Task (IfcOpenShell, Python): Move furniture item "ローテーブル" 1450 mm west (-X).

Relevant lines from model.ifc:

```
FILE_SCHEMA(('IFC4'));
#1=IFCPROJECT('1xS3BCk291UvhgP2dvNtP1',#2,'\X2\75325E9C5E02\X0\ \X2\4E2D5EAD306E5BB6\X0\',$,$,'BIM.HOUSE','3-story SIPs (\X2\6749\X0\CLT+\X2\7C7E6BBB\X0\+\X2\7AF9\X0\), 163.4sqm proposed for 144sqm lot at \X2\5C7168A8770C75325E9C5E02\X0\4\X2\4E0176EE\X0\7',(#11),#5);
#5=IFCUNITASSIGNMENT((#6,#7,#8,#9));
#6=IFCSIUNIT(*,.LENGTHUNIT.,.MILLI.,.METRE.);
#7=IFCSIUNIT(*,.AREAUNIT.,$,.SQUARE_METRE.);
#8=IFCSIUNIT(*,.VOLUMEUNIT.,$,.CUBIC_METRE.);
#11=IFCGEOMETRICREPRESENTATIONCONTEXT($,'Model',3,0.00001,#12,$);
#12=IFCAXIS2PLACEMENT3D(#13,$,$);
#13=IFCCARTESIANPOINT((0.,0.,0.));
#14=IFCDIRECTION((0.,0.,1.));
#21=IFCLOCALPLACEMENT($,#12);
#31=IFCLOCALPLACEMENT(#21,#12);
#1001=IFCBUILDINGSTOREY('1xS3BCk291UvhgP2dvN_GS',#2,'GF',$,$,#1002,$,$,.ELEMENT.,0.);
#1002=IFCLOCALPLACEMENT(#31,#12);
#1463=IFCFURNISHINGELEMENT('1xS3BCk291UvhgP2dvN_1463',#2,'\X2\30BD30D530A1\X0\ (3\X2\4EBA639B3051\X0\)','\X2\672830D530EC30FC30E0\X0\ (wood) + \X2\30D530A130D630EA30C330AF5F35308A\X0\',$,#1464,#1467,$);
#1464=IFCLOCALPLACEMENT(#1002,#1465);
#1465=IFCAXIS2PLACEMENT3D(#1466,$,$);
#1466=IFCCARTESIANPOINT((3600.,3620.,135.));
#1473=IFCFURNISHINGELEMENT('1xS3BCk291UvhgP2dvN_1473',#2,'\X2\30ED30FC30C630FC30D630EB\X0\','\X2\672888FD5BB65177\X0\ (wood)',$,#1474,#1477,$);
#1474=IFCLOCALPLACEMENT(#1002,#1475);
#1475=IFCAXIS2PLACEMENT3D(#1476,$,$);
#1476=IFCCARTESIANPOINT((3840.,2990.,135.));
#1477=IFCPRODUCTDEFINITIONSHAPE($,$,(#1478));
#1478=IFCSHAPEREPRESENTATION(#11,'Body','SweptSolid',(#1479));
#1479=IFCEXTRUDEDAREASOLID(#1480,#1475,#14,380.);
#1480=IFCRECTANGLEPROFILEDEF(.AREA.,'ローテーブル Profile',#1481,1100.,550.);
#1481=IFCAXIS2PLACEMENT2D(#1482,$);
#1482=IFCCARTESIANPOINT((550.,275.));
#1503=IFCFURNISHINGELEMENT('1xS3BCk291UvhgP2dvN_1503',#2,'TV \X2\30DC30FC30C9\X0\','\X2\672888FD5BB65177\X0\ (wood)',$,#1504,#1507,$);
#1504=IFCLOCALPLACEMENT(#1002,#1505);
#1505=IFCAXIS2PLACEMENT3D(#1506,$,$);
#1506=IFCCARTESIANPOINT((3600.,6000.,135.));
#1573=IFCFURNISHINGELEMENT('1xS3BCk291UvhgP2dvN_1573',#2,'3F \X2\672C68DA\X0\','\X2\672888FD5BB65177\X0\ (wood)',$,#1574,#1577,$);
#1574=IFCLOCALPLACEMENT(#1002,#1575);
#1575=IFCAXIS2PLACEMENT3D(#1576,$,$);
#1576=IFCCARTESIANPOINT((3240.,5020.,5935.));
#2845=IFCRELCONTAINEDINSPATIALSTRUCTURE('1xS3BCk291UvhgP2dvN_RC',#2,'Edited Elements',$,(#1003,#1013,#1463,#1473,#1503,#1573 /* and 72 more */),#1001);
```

```python
import ifcopenshell
import ifcopenshell.api.geometry
import ifcopenshell.util.placement
import ifcopenshell.util.unit

model = ifcopenshell.open("model.ifc")
unit_scale = ifcopenshell.util.unit.calculate_unit_scale(model)

item = model.by_guid("1xS3BCk291UvhgP2dvN_1473")
matrix = ifcopenshell.util.placement.get_local_placement(item.ObjectPlacement)
matrix[0, 3] -= 1.45 / unit_scale
ifcopenshell.api.geometry.edit_object_placement(model, product=item, matrix=matrix, is_si=False)

print(ifcopenshell.util.placement.get_local_placement(item.ObjectPlacement).round(3) + 0.0)

model.write("model_updated.ifc")
```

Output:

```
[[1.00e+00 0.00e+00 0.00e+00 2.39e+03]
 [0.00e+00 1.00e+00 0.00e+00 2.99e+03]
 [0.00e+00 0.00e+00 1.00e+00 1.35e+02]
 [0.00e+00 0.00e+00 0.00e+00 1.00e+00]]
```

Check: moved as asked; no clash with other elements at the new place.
